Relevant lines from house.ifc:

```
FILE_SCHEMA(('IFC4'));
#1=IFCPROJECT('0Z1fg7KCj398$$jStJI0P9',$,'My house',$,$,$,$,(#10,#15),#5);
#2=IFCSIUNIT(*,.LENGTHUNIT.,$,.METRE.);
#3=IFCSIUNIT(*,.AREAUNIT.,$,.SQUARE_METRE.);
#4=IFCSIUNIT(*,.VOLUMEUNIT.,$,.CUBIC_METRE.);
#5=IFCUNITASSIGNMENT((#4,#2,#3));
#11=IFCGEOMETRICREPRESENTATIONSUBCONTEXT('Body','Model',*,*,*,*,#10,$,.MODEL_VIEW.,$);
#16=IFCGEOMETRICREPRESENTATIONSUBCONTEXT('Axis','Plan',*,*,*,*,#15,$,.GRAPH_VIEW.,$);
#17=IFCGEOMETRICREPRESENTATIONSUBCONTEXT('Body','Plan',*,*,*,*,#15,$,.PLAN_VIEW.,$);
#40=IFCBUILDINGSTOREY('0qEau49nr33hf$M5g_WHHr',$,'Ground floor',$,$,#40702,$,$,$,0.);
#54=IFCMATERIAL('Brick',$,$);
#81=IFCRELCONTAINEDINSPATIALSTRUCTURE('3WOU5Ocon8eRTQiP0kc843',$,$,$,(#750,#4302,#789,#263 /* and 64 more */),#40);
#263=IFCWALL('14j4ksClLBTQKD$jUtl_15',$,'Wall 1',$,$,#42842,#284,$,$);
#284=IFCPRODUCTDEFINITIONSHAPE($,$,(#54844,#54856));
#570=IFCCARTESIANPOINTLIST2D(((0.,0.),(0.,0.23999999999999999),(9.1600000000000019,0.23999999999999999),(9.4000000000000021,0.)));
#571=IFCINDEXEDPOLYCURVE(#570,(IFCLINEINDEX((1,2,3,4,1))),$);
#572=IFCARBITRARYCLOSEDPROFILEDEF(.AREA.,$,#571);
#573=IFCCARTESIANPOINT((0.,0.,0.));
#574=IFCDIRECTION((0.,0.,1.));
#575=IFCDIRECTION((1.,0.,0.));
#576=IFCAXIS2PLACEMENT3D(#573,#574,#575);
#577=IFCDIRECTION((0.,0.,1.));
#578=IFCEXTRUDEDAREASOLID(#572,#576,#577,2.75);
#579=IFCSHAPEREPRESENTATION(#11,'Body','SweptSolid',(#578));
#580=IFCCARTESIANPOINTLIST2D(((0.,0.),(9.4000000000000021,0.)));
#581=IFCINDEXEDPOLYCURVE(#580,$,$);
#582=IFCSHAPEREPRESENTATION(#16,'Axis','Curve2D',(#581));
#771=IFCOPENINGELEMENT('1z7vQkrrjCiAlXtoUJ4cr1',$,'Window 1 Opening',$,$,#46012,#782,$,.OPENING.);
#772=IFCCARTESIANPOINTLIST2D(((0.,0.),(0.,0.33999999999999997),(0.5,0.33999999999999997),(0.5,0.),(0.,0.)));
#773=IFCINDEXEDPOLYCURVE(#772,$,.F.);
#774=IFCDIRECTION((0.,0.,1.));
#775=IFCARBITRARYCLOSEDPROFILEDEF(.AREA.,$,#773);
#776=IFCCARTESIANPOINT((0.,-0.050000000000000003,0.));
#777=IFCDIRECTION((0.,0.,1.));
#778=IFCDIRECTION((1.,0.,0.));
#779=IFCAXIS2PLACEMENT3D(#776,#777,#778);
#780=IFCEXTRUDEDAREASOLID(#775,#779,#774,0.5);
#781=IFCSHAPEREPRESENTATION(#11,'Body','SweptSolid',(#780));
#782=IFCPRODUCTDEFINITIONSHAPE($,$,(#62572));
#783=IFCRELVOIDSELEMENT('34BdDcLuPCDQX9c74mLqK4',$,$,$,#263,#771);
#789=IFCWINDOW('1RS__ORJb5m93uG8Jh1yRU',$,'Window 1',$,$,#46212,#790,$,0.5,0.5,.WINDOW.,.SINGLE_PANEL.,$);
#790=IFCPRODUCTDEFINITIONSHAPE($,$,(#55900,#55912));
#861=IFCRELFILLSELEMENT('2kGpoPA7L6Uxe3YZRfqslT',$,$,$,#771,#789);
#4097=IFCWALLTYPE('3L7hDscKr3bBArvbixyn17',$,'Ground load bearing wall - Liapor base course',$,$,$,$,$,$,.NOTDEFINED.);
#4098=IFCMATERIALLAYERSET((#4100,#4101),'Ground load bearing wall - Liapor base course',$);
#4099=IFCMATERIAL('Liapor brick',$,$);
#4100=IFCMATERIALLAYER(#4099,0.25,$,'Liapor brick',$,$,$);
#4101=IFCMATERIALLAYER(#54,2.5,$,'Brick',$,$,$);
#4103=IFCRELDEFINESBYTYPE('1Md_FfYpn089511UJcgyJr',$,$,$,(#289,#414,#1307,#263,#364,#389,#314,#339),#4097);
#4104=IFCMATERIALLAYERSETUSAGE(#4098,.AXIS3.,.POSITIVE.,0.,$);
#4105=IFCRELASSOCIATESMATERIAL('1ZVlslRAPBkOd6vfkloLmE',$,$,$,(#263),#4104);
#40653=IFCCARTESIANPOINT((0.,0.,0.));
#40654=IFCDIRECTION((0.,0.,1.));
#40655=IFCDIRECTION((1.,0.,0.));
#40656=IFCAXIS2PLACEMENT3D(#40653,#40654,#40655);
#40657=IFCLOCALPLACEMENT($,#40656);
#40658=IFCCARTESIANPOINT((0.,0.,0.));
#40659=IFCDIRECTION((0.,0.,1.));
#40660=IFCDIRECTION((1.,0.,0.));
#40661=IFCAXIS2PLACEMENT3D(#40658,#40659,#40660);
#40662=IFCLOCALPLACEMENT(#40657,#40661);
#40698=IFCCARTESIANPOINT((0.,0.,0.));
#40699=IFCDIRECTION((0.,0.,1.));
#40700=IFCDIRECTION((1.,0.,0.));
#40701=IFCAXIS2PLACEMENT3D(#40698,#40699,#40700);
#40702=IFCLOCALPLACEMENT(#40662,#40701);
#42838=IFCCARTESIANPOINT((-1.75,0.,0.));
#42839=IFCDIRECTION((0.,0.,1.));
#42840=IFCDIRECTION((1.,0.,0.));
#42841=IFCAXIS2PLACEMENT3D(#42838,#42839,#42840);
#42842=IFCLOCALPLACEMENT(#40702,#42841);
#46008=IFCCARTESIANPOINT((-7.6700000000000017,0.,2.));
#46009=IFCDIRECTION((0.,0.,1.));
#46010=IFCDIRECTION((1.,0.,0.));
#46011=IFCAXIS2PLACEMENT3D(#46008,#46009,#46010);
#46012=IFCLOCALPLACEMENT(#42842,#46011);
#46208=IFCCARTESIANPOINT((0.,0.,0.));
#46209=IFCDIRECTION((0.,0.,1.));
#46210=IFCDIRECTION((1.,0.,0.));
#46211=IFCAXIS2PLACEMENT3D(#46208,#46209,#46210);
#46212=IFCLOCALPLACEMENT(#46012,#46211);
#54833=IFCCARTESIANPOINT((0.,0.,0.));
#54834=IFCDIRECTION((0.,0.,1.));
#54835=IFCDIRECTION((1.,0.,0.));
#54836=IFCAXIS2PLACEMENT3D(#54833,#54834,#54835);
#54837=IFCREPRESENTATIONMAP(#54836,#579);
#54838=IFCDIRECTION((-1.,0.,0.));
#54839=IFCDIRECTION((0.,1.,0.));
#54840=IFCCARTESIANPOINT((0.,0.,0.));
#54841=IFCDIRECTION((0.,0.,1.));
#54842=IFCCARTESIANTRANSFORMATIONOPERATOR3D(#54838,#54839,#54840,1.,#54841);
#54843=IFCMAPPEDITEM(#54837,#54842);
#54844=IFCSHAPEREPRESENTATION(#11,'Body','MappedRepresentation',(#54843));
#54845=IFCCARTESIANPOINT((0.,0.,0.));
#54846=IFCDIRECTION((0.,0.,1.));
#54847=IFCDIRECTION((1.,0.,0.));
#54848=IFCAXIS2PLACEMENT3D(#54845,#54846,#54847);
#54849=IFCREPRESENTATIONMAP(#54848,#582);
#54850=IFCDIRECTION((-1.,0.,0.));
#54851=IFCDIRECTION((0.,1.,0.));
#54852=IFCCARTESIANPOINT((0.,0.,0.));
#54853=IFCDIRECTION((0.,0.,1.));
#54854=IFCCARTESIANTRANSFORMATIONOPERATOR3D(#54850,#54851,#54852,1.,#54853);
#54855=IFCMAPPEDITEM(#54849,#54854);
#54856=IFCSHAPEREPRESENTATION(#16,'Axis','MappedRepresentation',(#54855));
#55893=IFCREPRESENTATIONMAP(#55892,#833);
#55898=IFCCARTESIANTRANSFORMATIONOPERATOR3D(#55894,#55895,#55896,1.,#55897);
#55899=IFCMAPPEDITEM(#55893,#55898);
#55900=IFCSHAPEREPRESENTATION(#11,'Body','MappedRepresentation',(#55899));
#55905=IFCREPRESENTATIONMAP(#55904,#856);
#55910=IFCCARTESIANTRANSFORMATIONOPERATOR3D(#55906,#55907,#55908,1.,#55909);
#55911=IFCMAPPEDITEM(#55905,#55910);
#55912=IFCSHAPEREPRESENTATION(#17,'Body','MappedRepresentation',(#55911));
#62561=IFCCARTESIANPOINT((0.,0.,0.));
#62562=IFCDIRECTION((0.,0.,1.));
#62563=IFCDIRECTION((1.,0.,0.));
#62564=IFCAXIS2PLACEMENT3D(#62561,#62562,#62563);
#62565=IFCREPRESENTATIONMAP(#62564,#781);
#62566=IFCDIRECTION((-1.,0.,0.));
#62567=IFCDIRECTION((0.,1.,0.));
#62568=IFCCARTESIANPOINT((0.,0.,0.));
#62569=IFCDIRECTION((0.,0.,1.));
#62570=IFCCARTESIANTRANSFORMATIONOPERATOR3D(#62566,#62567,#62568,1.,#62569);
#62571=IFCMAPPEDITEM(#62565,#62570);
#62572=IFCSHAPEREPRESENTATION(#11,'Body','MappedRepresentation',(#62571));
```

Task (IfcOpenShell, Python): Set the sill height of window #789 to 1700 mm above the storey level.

```python
import numpy as np
import ifcopenshell
import ifcopenshell.api.geometry
import ifcopenshell.geom
import ifcopenshell.util.element
import ifcopenshell.util.placement
import ifcopenshell.util.shape
import ifcopenshell.util.unit

model = ifcopenshell.open("house.ifc")
unit_scale = ifcopenshell.util.unit.calculate_unit_scale(model)

window = model.by_guid("1RS__ORJb5m93uG8Jh1yRU")
opening = window.FillsVoids[0].RelatingOpeningElement
storey = ifcopenshell.util.element.get_container(window, ifc_class="IfcBuildingStorey")
level = ifcopenshell.util.placement.get_local_placement(storey.ObjectPlacement)[2, 3]

# The opening's origin need not be at the sill, so measure its lowest point.
shape = ifcopenshell.geom.create_shape(ifcopenshell.geom.settings(), opening)
bottom = ifcopenshell.util.shape.get_shape_bottom_elevation(shape, shape.geometry) / unit_scale
dz = level + 1.7 / unit_scale - bottom

shift = np.array([0.0, 0.0, dz])
# The window is placed relative to its opening, so it follows when the opening moves.
matrix = ifcopenshell.util.placement.get_local_placement(opening.ObjectPlacement)
matrix[:3, 3] += shift
ifcopenshell.api.geometry.edit_object_placement(
    model, product=opening, matrix=matrix, is_si=False, should_transform_children=True
)

print(f"moved by {dz * unit_scale:+.3f} m")

model.write("house_rev.ifc")
```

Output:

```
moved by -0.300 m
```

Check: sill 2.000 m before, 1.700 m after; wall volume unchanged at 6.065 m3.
